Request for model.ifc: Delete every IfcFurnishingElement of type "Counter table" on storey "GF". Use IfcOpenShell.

First a look at what the model holds.

```python
import ifcopenshell
import ifcopenshell.util.element

model = ifcopenshell.open("model.ifc")
print(model.schema)
storey = next(s for s in model.by_type("IfcBuildingStorey") if s.Name == "GF")
furniture = [e for e in ifcopenshell.util.element.get_decomposition(storey) if e.is_a("IfcFurnishingElement")]
seen = {}
for e in furniture:
    element_type = ifcopenshell.util.element.get_type(e)
    name = element_type.Name if element_type not in (None, e) else None
    seen[name] = seen.get(name, 0) + 1
for name, count in sorted(seen.items(), key=str):
    print(count, "x", name)
```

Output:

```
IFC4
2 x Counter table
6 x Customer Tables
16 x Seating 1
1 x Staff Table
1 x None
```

```python
import ifcopenshell
import ifcopenshell.api.root
import ifcopenshell.util.element

model = ifcopenshell.open("model.ifc")

storey = next(s for s in model.by_type("IfcBuildingStorey") if s.Name == "GF")
furniture = [e for e in ifcopenshell.util.element.get_decomposition(storey) if e.is_a("IfcFurnishingElement")]
targets = [e for e in furniture if (t := ifcopenshell.util.element.get_type(e)) not in (None, e) and t.Name == "Counter table"]

for e in targets:
    ifcopenshell.api.root.remove_product(model, product=e)
print(len(targets), "removed")

model.write("model_updated.ifc")
```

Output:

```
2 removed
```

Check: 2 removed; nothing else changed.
